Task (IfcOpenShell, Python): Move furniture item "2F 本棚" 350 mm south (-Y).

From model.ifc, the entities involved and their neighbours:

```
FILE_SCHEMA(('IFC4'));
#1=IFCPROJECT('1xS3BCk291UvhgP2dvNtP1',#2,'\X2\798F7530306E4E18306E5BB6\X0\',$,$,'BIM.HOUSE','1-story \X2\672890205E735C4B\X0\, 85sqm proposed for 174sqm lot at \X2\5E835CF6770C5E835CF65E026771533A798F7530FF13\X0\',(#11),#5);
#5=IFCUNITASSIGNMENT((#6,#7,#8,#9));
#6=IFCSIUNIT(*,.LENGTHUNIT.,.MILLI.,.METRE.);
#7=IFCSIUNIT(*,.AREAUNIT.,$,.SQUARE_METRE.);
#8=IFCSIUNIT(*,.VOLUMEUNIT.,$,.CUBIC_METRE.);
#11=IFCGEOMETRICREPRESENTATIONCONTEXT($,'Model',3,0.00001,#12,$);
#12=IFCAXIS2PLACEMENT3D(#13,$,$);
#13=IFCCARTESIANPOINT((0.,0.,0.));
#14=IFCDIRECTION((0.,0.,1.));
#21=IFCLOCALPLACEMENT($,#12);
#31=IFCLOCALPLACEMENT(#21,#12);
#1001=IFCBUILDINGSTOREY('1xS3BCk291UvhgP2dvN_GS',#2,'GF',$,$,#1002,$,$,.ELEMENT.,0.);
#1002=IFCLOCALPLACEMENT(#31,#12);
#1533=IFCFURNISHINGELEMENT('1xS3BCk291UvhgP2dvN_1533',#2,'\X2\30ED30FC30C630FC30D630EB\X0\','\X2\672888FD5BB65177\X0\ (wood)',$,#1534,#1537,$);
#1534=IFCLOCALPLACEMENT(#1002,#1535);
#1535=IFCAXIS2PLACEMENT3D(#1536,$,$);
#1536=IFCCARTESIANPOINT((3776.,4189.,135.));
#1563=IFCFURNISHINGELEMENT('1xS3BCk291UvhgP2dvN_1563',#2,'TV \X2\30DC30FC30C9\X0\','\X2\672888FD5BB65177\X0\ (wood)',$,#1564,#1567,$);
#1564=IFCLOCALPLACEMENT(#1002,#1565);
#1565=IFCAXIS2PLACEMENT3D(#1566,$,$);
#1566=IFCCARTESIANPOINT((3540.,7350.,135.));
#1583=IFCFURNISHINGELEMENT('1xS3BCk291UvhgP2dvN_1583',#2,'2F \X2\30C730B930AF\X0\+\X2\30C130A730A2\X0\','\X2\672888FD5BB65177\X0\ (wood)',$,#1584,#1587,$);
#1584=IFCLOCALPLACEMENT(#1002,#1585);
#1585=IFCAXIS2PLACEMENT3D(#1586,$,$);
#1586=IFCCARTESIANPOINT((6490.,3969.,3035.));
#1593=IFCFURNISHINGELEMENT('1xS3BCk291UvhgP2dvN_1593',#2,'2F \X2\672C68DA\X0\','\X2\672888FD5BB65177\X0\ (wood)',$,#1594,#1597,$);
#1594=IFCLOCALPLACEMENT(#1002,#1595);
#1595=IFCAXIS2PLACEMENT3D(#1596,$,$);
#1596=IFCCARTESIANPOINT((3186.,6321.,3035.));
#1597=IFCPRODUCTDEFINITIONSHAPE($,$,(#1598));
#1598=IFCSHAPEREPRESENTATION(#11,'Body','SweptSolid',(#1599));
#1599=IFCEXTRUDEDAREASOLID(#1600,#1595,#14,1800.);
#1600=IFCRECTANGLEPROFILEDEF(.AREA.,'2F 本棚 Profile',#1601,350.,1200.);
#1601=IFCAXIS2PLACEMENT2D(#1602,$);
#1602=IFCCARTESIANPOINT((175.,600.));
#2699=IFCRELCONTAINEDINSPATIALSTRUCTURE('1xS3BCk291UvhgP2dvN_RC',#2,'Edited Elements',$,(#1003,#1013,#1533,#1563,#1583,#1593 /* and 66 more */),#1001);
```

```python
import ifcopenshell
import ifcopenshell.api.geometry
import ifcopenshell.util.placement
import ifcopenshell.util.unit

model = ifcopenshell.open("model.ifc")
unit_scale = ifcopenshell.util.unit.calculate_unit_scale(model)

item = model.by_id(1593)
matrix = ifcopenshell.util.placement.get_local_placement(item.ObjectPlacement)
matrix[1, 3] -= 0.35 / unit_scale
ifcopenshell.api.geometry.edit_object_placement(model, product=item, matrix=matrix, is_si=False)

print(ifcopenshell.util.placement.get_local_placement(item.ObjectPlacement).round(3) + 0.0)

model.write("model_edited.ifc")
```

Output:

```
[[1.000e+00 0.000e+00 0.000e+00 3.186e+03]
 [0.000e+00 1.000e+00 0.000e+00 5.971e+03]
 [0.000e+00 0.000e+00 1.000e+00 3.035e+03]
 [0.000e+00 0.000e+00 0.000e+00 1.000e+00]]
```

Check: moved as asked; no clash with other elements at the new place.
